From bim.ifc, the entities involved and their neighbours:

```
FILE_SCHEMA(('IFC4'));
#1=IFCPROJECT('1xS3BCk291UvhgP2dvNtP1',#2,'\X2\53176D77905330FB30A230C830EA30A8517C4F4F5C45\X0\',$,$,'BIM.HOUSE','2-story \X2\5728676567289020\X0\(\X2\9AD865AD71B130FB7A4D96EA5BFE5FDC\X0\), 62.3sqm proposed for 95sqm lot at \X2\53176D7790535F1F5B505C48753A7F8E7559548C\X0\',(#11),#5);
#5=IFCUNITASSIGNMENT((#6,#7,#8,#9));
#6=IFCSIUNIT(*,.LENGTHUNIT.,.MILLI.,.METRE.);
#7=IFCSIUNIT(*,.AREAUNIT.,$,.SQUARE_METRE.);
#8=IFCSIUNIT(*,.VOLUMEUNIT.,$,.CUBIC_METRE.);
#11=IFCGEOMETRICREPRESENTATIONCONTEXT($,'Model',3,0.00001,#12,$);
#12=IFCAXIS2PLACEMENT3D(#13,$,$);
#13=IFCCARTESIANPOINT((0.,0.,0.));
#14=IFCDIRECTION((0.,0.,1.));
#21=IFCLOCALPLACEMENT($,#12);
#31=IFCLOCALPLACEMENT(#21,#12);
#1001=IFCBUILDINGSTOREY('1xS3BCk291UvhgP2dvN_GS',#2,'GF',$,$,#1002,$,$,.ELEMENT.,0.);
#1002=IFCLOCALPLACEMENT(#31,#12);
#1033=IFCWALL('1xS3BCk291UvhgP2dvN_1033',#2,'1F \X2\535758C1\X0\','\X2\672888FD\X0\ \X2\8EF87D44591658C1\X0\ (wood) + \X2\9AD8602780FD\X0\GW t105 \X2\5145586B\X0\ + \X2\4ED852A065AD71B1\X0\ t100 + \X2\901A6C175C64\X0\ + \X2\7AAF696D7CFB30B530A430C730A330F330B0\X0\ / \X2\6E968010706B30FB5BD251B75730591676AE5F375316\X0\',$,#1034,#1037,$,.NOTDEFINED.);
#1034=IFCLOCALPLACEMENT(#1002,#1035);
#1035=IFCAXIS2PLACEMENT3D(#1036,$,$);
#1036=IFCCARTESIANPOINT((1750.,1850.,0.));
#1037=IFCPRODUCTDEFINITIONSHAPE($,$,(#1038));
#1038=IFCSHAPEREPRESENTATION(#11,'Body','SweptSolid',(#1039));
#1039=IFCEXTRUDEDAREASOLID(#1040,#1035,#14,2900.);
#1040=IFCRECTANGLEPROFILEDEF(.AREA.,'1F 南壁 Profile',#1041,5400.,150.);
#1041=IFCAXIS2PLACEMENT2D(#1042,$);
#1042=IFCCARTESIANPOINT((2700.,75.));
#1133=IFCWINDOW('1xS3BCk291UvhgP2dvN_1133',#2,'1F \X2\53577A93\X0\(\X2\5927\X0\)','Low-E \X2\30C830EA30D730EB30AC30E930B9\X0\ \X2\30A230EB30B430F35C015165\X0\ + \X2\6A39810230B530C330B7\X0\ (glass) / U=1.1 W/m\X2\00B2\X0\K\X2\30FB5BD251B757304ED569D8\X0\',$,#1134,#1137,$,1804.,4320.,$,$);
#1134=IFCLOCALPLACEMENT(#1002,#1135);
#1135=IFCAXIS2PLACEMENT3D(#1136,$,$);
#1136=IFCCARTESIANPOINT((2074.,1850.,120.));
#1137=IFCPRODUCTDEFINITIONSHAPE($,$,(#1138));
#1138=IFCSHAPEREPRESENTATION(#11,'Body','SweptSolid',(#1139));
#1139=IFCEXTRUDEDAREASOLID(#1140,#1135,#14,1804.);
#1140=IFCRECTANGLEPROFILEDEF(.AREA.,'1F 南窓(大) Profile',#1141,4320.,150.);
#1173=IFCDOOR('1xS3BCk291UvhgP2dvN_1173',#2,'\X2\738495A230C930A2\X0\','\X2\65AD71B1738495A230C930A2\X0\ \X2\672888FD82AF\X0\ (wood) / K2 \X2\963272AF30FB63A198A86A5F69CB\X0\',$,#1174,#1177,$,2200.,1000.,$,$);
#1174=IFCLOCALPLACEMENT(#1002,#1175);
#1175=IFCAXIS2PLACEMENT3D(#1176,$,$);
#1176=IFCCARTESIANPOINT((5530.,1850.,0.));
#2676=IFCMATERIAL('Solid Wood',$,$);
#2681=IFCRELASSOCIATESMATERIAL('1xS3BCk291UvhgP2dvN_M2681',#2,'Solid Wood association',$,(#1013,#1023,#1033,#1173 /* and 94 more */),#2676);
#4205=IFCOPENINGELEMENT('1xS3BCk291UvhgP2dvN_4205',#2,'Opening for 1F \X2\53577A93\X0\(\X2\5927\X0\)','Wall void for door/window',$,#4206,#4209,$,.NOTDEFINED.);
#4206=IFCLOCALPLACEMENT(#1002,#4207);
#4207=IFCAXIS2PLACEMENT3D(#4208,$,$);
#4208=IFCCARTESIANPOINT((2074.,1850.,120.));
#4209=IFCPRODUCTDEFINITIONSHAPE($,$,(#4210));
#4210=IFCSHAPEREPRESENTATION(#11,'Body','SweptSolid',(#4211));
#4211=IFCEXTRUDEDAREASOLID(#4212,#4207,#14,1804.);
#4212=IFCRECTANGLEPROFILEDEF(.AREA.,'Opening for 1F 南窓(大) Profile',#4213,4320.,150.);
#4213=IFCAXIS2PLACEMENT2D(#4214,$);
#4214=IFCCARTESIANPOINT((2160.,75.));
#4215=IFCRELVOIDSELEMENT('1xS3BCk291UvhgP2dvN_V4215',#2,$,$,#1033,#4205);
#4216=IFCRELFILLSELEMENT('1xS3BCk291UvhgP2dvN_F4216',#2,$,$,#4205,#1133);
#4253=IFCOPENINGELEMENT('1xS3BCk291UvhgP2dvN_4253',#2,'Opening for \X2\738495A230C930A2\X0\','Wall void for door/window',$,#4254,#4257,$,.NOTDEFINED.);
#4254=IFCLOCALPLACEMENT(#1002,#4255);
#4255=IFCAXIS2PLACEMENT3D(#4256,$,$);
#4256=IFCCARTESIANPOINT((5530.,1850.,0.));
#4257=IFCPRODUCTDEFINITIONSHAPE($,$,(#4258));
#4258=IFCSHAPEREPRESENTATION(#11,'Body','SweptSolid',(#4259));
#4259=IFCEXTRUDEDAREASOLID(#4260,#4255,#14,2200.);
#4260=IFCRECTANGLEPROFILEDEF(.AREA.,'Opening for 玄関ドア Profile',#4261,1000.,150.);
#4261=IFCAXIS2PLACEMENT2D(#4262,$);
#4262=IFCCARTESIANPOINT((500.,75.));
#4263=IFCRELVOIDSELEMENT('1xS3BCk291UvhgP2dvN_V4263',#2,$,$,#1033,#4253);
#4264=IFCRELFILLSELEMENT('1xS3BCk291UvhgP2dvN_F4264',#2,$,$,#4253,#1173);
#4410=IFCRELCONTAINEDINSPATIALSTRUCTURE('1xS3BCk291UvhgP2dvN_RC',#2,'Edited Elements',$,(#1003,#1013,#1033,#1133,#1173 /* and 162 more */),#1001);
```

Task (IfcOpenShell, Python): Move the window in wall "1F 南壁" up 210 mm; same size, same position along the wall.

```python
import numpy as np
import ifcopenshell
import ifcopenshell.api.geometry
import ifcopenshell.util.placement
import ifcopenshell.util.unit

model = ifcopenshell.open("bim.ifc")
unit_scale = ifcopenshell.util.unit.calculate_unit_scale(model)

window = model.by_guid("1xS3BCk291UvhgP2dvN_1133")
opening = window.FillsVoids[0].RelatingOpeningElement
dz = 210.0

shift = np.array([0.0, 0.0, dz])
# The window is not placed relative to its opening, so move both.
for product in (opening, window):
    matrix = ifcopenshell.util.placement.get_local_placement(product.ObjectPlacement)
    matrix[:3, 3] += shift
    ifcopenshell.api.geometry.edit_object_placement(model, product=product, matrix=matrix, is_si=False)

print(f"moved by {dz * unit_scale:+.3f} m")

model.write("bim_rev.ifc")
```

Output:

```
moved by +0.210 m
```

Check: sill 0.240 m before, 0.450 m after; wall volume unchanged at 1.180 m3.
